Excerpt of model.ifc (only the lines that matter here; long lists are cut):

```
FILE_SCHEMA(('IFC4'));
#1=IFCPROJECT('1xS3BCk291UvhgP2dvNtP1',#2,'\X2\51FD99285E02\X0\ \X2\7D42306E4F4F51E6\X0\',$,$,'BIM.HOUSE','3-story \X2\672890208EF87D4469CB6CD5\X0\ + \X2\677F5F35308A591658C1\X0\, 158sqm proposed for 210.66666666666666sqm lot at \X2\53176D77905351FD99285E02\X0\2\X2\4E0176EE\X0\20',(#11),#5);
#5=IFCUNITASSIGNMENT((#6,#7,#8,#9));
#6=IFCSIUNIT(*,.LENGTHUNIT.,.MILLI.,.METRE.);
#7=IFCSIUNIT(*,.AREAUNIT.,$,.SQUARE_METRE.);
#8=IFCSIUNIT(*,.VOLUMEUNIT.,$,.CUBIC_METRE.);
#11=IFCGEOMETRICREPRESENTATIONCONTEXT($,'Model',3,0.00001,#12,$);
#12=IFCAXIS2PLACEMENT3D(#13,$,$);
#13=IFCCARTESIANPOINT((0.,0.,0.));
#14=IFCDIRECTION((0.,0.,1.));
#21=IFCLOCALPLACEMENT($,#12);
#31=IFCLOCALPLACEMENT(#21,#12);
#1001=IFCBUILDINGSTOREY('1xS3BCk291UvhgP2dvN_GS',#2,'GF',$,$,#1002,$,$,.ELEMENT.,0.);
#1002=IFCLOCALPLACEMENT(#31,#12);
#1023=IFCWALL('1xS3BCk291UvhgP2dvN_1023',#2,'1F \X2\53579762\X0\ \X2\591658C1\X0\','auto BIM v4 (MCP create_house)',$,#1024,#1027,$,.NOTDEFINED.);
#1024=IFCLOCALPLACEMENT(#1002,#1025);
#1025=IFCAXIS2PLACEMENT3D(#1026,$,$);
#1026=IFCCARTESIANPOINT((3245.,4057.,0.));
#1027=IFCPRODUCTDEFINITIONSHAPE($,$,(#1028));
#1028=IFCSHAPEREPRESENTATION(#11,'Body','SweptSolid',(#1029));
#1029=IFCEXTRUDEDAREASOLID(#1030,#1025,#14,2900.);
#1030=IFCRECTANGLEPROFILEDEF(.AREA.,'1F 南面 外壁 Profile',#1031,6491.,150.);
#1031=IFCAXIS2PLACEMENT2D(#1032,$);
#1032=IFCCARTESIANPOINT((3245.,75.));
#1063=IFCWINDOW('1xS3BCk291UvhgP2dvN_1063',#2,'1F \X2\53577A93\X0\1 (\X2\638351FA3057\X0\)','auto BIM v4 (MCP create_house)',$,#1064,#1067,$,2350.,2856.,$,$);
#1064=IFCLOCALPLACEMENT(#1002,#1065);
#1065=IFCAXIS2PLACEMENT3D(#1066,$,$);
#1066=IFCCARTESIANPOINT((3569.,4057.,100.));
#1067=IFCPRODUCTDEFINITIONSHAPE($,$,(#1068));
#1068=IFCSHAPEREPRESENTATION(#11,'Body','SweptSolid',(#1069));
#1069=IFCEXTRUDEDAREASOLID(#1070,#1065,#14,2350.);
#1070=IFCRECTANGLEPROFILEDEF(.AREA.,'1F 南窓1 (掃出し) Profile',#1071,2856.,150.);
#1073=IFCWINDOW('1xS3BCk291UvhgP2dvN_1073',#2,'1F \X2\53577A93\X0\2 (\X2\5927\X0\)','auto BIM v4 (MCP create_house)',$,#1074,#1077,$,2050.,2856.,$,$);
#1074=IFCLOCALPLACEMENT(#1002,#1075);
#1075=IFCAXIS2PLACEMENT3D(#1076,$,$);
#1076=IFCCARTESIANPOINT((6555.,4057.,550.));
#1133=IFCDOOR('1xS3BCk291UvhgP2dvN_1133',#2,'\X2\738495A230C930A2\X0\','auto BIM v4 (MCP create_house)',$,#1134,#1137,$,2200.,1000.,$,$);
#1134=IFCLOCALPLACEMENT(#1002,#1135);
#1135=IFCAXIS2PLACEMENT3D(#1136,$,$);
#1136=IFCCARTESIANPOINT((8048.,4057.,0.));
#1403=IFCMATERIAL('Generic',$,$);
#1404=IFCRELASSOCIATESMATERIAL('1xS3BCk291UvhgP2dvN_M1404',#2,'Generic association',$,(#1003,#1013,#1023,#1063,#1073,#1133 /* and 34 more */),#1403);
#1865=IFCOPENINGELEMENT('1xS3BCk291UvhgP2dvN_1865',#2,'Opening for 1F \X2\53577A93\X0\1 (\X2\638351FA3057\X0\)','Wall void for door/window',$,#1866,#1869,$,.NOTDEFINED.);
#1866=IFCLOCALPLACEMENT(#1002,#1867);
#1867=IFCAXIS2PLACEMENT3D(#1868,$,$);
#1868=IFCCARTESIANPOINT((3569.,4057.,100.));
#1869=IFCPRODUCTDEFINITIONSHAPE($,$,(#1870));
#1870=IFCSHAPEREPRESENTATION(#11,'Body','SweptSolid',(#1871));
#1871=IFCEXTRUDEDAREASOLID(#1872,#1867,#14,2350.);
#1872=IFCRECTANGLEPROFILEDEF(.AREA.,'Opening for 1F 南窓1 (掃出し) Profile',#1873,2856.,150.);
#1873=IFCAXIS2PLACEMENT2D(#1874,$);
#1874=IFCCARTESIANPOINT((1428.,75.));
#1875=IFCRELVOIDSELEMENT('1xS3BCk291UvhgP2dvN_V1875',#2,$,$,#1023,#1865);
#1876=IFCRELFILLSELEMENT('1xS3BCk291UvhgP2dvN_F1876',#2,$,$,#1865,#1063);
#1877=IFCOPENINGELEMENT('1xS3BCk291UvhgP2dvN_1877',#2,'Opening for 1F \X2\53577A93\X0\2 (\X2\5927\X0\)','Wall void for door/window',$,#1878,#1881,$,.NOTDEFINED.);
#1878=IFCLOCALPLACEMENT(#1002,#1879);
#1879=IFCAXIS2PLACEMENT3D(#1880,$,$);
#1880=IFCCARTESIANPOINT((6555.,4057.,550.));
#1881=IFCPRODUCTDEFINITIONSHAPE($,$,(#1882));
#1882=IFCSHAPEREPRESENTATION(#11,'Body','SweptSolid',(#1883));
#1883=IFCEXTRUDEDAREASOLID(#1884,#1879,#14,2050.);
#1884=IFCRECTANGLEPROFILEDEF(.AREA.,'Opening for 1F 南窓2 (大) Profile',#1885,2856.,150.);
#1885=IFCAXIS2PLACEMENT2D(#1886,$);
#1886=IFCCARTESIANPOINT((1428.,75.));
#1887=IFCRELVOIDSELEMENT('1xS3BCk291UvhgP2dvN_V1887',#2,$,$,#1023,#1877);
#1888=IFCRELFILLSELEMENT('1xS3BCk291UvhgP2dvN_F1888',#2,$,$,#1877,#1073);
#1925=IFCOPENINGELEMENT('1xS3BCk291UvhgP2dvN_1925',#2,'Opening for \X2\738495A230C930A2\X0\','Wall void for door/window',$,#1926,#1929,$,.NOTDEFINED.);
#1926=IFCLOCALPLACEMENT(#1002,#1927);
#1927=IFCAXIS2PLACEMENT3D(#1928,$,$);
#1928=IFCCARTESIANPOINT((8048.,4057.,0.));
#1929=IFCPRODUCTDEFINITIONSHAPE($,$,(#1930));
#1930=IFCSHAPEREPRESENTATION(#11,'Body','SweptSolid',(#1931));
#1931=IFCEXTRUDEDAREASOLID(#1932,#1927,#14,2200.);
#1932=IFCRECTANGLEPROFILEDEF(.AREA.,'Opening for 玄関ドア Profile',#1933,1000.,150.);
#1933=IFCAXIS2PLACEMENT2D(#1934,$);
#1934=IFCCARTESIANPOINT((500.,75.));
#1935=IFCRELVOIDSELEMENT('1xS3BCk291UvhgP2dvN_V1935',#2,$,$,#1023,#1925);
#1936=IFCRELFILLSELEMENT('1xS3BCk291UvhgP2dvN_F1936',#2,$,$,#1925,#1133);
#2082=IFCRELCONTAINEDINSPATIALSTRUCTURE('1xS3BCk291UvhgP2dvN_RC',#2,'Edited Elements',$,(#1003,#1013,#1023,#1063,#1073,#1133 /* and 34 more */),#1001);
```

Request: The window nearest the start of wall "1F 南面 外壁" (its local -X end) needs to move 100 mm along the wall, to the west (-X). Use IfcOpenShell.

```python
import ifcopenshell
import ifcopenshell.api.geometry
import ifcopenshell.util.placement
import ifcopenshell.util.unit

model = ifcopenshell.open("model.ifc")
unit_scale = ifcopenshell.util.unit.calculate_unit_scale(model)

window = model.by_id(1063)
opening = window.FillsVoids[0].RelatingOpeningElement
wall = opening.VoidsElements[0].RelatingBuildingElement

wall_matrix = ifcopenshell.util.placement.get_local_placement(wall.ObjectPlacement)
shift = wall_matrix[:3, 0] * -0.1 / unit_scale
before = ifcopenshell.util.placement.get_local_placement(window.ObjectPlacement)[:3, 3].copy()

# The window is not placed relative to its opening, so move both.
for product in (opening, window):
    matrix = ifcopenshell.util.placement.get_local_placement(product.ObjectPlacement)
    matrix[:3, 3] += shift
    ifcopenshell.api.geometry.edit_object_placement(model, product=product, matrix=matrix, is_si=False)

after = ifcopenshell.util.placement.get_local_placement(window.ObjectPlacement)[:3, 3]
print("window moved by", (after - before).round(3) + 0.0)

model.write("model-out.ifc")
```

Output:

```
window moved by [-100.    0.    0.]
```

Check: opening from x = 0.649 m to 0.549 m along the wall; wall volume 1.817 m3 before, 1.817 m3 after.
